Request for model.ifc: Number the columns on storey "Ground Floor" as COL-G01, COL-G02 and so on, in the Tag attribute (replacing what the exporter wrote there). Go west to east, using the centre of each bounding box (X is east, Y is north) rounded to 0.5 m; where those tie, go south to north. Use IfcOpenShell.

First a look at what the model holds.

```python
import ifcopenshell
import ifcopenshell.util.element
import ifcopenshell.util.placement

model = ifcopenshell.open("model.ifc")
print(model.schema)
storey = next(s for s in model.by_type("IfcBuildingStorey") if s.Name == "Ground Floor")
columns = [e for e in ifcopenshell.util.element.get_decomposition(storey) if e.is_a("IfcColumn")]
for e in sorted(columns, key=lambda e: e.id()):
    origin = ifcopenshell.util.placement.get_local_placement(e.ObjectPlacement)[:3, 3]
    print(e.id(), e.Tag, e.Name, origin.round(2) + 0.0, sep=" | ")
```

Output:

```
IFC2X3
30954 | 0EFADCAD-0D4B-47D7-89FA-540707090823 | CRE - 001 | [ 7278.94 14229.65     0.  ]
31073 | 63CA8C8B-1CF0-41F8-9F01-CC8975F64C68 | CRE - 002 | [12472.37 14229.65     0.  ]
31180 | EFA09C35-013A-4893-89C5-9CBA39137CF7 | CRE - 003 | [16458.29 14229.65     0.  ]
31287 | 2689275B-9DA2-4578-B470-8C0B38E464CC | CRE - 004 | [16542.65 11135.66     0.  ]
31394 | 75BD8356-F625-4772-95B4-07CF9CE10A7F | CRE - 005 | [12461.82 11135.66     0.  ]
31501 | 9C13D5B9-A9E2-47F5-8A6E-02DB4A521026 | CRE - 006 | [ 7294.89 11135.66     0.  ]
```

```python
import ifcopenshell
import ifcopenshell.geom
import ifcopenshell.util.element
import ifcopenshell.util.shape

model = ifcopenshell.open("model.ifc")
settings = ifcopenshell.geom.settings()
settings.set("use-world-coords", True)


def centre(element):
    shape = ifcopenshell.geom.create_shape(settings, element)
    return ifcopenshell.util.shape.get_bbox_centroid(shape.geometry)


storey = next(s for s in model.by_type("IfcBuildingStorey") if s.Name == "Ground Floor")
columns = [e for e in ifcopenshell.util.element.get_decomposition(storey) if e.is_a("IfcColumn")]

# Insertion points can sit at a corner or the storey origin, so sort by the geometry (in metres).
centres = {e: centre(e) for e in columns}
columns.sort(key=lambda e: (round(centres[e][0] / 0.5), centres[e][1]))

for i, e in enumerate(columns, start=1):
    number = f"COL-G{i:02d}"
    e.Tag = number
    print(e.id(), number)

model.write("model_edited.ifc")
```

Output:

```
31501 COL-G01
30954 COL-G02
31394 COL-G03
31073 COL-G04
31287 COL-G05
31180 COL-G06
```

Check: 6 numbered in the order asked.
